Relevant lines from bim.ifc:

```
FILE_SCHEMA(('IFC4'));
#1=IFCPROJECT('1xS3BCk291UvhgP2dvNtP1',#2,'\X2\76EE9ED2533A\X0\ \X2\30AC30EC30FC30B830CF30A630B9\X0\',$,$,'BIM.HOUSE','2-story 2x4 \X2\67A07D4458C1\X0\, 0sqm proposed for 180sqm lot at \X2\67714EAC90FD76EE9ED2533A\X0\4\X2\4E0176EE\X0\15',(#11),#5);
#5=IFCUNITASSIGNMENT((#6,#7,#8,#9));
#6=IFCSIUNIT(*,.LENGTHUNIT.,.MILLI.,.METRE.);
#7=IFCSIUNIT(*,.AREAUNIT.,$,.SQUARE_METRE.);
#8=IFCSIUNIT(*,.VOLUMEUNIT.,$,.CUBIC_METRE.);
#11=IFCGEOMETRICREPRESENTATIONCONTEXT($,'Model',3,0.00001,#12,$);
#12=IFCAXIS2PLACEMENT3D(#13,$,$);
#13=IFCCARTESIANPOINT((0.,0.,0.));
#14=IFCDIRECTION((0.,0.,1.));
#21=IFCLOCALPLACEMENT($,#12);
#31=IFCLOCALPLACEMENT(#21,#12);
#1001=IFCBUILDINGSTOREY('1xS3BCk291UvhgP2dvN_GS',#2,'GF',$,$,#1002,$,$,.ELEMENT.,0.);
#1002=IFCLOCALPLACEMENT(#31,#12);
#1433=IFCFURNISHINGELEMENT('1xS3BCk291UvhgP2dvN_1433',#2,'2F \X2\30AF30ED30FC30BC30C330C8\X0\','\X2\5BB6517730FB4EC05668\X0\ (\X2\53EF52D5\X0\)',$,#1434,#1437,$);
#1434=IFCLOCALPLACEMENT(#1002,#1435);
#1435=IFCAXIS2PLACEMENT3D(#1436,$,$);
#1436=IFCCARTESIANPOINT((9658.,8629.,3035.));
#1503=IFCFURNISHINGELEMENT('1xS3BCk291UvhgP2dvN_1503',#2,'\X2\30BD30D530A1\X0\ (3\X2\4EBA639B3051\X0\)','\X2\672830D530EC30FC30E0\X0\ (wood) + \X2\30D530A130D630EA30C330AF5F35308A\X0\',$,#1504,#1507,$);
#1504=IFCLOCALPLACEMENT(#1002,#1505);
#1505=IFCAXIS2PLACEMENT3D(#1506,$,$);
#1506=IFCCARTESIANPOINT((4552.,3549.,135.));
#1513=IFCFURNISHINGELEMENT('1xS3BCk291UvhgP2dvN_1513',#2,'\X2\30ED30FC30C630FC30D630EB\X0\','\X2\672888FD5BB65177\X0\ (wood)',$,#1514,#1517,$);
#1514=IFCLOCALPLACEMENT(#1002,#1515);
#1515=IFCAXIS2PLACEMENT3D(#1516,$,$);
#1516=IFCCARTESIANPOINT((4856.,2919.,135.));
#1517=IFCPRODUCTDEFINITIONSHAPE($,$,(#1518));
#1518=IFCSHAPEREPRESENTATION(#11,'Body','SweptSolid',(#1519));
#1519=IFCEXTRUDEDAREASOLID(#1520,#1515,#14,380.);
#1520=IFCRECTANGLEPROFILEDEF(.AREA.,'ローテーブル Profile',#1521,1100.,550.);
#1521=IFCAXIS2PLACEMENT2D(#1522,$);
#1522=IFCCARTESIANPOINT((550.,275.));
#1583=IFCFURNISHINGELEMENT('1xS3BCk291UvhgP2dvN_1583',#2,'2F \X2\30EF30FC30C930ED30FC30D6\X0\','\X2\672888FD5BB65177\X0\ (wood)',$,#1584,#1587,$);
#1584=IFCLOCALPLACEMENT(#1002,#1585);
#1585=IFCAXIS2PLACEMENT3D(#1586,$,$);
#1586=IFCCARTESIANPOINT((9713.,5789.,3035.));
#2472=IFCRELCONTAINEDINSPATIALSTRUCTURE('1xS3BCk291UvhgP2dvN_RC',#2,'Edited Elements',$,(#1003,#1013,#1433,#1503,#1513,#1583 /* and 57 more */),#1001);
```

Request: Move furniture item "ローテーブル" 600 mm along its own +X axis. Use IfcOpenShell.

```python
import ifcopenshell
import ifcopenshell.api.geometry
import ifcopenshell.util.placement
import ifcopenshell.util.unit

model = ifcopenshell.open("bim.ifc")
unit_scale = ifcopenshell.util.unit.calculate_unit_scale(model)

item = model.by_id(1513)
matrix = ifcopenshell.util.placement.get_local_placement(item.ObjectPlacement)
matrix[:3, 3] += matrix[:3, 0] * 0.6 / unit_scale
ifcopenshell.api.geometry.edit_object_placement(model, product=item, matrix=matrix, is_si=False)

print(ifcopenshell.util.placement.get_local_placement(item.ObjectPlacement).round(3) + 0.0)

model.write("bim_updated.ifc")
```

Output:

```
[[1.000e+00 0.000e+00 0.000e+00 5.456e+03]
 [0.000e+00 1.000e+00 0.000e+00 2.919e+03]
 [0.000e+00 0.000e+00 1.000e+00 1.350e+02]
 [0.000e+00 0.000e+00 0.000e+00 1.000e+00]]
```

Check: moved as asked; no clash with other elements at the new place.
